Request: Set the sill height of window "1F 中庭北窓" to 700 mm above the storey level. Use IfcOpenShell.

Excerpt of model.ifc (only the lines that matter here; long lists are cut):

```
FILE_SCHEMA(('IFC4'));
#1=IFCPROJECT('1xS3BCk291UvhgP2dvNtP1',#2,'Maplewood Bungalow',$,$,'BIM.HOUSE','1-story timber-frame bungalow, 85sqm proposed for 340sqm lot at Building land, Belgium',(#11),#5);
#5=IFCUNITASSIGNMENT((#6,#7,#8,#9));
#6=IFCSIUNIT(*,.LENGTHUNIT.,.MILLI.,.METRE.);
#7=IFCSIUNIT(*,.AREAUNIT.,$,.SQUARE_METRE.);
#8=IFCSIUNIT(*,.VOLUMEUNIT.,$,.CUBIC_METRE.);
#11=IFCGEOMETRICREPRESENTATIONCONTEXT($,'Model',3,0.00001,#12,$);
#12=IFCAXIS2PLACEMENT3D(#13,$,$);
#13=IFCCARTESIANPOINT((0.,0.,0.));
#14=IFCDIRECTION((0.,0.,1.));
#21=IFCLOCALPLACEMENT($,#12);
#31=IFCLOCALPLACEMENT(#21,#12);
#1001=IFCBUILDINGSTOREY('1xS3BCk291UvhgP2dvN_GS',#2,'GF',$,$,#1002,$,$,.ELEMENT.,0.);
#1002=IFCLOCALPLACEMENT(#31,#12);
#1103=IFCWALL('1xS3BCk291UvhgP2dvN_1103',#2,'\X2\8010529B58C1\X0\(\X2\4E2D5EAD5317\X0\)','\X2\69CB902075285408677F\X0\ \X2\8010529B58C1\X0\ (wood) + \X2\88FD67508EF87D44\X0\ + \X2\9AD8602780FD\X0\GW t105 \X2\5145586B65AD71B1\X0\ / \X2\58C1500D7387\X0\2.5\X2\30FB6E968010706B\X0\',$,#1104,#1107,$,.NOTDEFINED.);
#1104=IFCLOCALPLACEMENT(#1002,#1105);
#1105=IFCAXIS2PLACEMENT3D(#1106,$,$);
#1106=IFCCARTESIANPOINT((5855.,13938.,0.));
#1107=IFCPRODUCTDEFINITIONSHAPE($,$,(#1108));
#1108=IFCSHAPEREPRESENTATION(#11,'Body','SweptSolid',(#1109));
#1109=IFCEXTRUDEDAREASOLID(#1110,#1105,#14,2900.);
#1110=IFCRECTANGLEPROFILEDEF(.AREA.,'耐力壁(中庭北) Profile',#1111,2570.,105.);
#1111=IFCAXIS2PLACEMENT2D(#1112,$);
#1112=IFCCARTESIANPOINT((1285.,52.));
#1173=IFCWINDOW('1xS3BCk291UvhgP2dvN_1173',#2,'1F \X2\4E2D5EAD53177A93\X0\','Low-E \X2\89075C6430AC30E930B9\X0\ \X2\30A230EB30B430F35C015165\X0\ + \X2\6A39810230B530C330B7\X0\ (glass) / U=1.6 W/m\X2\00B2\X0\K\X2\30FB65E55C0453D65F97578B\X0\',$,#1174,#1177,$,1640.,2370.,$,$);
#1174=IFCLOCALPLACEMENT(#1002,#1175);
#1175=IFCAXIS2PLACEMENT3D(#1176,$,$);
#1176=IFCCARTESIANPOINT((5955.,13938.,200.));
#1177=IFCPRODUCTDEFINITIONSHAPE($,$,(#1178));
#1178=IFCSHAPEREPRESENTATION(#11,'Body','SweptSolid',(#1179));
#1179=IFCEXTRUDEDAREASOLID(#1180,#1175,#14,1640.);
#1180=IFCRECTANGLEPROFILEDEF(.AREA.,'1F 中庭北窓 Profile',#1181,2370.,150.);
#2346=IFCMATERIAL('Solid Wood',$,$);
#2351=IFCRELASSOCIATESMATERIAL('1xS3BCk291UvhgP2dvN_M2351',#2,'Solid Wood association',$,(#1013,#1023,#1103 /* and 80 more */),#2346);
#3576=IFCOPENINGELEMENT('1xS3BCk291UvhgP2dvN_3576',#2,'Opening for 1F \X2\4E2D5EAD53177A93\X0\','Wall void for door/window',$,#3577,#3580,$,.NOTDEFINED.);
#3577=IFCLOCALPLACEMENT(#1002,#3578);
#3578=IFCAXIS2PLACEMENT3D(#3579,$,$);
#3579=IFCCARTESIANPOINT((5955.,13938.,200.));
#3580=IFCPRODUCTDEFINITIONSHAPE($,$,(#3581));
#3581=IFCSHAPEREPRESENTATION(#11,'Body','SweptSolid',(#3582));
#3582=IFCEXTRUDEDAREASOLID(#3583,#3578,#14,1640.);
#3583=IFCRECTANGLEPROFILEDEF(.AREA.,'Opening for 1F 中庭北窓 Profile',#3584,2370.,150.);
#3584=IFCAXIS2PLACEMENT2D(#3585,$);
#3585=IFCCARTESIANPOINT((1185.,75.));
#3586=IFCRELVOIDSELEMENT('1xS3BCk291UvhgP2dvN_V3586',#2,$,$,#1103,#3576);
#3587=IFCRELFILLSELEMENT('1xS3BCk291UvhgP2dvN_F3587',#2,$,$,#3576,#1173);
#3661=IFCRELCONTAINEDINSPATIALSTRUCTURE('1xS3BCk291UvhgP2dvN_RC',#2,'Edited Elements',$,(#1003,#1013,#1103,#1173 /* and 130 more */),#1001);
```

```python
import numpy as np
import ifcopenshell
import ifcopenshell.api.geometry
import ifcopenshell.geom
import ifcopenshell.util.element
import ifcopenshell.util.placement
import ifcopenshell.util.shape
import ifcopenshell.util.unit

model = ifcopenshell.open("model.ifc")
unit_scale = ifcopenshell.util.unit.calculate_unit_scale(model)

window = model.by_guid("1xS3BCk291UvhgP2dvN_1173")
opening = window.FillsVoids[0].RelatingOpeningElement
storey = ifcopenshell.util.element.get_container(window, ifc_class="IfcBuildingStorey")
level = ifcopenshell.util.placement.get_local_placement(storey.ObjectPlacement)[2, 3]

# The opening's origin need not be at the sill, so measure its lowest point.
shape = ifcopenshell.geom.create_shape(ifcopenshell.geom.settings(), opening)
bottom = ifcopenshell.util.shape.get_shape_bottom_elevation(shape, shape.geometry) / unit_scale
dz = level + 0.7 / unit_scale - bottom

shift = np.array([0.0, 0.0, dz])
# The window is not placed relative to its opening, so move both.
for product in (opening, window):
    matrix = ifcopenshell.util.placement.get_local_placement(product.ObjectPlacement)
    matrix[:3, 3] += shift
    ifcopenshell.api.geometry.edit_object_placement(model, product=product, matrix=matrix, is_si=False)

print(f"moved by {dz * unit_scale:+.3f} m")

model.write("model_updated.ifc")
```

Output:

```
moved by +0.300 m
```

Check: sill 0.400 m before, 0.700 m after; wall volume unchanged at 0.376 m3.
